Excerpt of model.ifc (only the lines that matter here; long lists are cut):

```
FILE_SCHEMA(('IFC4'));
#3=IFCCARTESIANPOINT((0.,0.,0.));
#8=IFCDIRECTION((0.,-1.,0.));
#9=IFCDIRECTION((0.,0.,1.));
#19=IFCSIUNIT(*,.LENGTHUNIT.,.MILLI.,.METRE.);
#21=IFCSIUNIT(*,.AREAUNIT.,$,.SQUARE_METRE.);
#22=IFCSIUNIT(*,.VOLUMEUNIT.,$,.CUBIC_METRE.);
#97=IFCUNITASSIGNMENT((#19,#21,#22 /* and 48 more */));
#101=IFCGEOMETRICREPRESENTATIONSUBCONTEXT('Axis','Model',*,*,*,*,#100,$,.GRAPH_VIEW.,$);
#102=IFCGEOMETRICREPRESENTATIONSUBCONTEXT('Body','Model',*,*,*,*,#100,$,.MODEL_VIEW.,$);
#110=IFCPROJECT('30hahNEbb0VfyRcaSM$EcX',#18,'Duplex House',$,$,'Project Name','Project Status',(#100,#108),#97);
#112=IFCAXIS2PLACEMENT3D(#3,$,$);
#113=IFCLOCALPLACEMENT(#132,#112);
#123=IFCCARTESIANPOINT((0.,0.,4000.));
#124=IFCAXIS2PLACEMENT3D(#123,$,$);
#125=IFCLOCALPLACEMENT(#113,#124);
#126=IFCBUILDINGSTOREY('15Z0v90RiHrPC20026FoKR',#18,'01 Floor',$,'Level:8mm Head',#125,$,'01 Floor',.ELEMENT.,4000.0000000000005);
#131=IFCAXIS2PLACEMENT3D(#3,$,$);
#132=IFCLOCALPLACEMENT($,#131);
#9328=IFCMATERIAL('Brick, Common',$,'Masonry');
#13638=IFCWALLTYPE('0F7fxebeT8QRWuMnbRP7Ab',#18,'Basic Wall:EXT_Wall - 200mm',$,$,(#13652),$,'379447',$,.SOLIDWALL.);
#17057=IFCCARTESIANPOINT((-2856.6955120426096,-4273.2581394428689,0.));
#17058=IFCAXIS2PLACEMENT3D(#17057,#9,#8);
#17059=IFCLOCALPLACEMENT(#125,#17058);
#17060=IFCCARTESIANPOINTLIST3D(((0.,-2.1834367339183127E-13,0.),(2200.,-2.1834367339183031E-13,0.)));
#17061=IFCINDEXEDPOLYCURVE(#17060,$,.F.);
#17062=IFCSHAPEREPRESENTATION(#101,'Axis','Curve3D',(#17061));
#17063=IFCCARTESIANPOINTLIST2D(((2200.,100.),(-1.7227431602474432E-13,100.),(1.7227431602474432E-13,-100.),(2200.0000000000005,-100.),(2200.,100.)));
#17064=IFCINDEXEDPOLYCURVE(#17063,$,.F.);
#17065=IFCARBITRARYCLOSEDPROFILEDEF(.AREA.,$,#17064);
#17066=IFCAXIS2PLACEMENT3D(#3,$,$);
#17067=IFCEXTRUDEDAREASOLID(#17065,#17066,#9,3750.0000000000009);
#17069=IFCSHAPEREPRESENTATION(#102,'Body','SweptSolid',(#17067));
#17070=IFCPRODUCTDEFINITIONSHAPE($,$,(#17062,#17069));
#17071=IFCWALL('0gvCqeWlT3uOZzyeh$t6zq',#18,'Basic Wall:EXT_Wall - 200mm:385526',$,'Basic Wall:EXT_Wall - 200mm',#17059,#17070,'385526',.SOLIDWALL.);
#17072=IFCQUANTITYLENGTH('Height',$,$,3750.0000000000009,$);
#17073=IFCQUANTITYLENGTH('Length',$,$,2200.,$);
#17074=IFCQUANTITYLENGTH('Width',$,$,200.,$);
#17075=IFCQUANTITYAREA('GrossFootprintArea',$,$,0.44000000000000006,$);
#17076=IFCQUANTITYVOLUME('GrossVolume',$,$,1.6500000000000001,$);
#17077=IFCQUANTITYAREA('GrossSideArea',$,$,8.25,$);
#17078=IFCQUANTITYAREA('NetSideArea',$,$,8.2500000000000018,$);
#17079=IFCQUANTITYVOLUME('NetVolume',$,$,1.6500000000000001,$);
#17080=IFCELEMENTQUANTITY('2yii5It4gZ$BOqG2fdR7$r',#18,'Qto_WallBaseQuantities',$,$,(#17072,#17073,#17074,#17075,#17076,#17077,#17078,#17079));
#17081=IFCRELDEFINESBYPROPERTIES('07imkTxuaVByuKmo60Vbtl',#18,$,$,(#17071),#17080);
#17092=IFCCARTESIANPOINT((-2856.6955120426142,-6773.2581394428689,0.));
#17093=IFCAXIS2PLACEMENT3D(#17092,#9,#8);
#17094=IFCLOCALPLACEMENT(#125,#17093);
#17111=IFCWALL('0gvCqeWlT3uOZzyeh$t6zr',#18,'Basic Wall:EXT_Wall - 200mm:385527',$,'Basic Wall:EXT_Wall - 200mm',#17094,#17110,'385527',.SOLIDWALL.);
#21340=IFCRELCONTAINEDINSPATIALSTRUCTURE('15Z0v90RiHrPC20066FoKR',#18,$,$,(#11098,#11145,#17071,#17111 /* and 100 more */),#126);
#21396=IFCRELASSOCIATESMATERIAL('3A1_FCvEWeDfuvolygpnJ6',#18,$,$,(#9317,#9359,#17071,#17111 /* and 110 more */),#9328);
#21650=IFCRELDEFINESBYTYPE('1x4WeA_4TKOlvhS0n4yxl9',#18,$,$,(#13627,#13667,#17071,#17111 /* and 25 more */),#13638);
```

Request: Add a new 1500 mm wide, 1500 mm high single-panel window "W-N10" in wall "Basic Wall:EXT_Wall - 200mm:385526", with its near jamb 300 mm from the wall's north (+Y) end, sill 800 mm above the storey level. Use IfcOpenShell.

```python
import numpy as np
import ifcopenshell
import ifcopenshell.api.feature
import ifcopenshell.api.geometry
import ifcopenshell.api.pset
import ifcopenshell.api.root
import ifcopenshell.api.spatial
import ifcopenshell.geom
import ifcopenshell.util.element
import ifcopenshell.util.placement
import ifcopenshell.util.representation
import ifcopenshell.util.shape
import ifcopenshell.util.unit

model = ifcopenshell.open("model.ifc")
unit_scale = ifcopenshell.util.unit.calculate_unit_scale(model)
area_scale = ifcopenshell.util.unit.calculate_unit_scale(model, "AREAUNIT")
volume_scale = ifcopenshell.util.unit.calculate_unit_scale(model, "VOLUMEUNIT")
settings = ifcopenshell.geom.settings()


def volume(element):
    """Net volume in cubic metres, openings subtracted."""
    shape = ifcopenshell.geom.create_shape(settings, element)
    return ifcopenshell.util.shape.get_volume(shape.geometry)


wall = model.by_guid("0gvCqeWlT3uOZzyeh$t6zq")
storey = ifcopenshell.util.element.get_container(wall, ifc_class="IfcBuildingStorey")
context = ifcopenshell.util.representation.get_context(model, "Model", "Body", "MODEL_VIEW")
before = volume(wall)

width, height, from_end, sill = 1.5, 1.5, 0.3, 0.8  # metres

# The wall runs along its own X axis, and the end named is its -X end.
wall_shape = ifcopenshell.geom.create_shape(settings, wall)
x, y, z = ifcopenshell.util.shape.get_vertices(wall_shape.geometry).T
start = x.min() + from_end
face, thickness = float(y.min()), float(y.max() - y.min())
wall_matrix = ifcopenshell.util.placement.get_local_placement(wall.ObjectPlacement)
level = ifcopenshell.util.placement.get_local_placement(storey.ObjectPlacement)[2, 3]


def in_wall(x, y):
    """Placement at x, y metres in the wall's axes, at sill height."""
    matrix = wall_matrix.copy()
    matrix[:, 3] = wall_matrix @ np.array([x / unit_scale, y / unit_scale, 0.0, 1.0])
    matrix[2, 3] = level + sill / unit_scale
    return matrix


# Opening: a box that overshoots both wall faces by 50 mm.
opening = ifcopenshell.api.root.create_entity(model, ifc_class="IfcOpeningElement", predefined_type="OPENING")
box = ifcopenshell.api.geometry.add_wall_representation(
    model, context=context, length=width, height=height, thickness=thickness + 0.1
)
ifcopenshell.api.geometry.assign_representation(model, product=opening, representation=box)
ifcopenshell.api.geometry.edit_object_placement(model, product=opening, matrix=in_wall(start, face - 0.05), is_si=False)
ifcopenshell.api.feature.add_feature(model, feature=opening, element=wall)

window = ifcopenshell.api.root.create_entity(model, ifc_class="IfcWindow", name="W-N10", predefined_type="WINDOW")
window.OverallWidth, window.OverallHeight = width / unit_scale, height / unit_scale
window.PartitioningType = "SINGLE_PANEL"
body = ifcopenshell.api.geometry.add_window_representation(
    model,
    context=context,
    overall_width=window.OverallWidth,
    overall_height=window.OverallHeight,
    partition_type="SINGLE_PANEL",
)
ifcopenshell.api.geometry.assign_representation(model, product=window, representation=body)
ifcopenshell.api.spatial.assign_container(model, products=[window], relating_structure=storey)
ifcopenshell.api.feature.add_filling(model, opening=opening, element=window)

# Centre the window in the wall's thickness.
ifcopenshell.api.geometry.edit_object_placement(model, product=window, matrix=in_wall(start, face), is_si=False)
window_shape = ifcopenshell.geom.create_shape(settings, window)
depth = ifcopenshell.util.shape.get_vertices(window_shape.geometry)[:, 1]
offset = face + thickness / 2 - (depth.min() + depth.max()) / 2
ifcopenshell.api.geometry.edit_object_placement(model, product=window, matrix=in_wall(start, offset), is_si=False)

after = volume(wall)

# Update the wall's stored quantities.
qto = model.by_id(ifcopenshell.util.element.get_pset(wall, "Qto_WallBaseQuantities", should_inherit=False)["id"])
ifcopenshell.api.pset.edit_qto(model, qto=qto, properties={
    "NetSideArea": after / thickness / area_scale,
    "NetVolume": after / volume_scale,
})

print(f"wall volume {before:.3f} -> {after:.3f} m3")

model.write("model_edited.ifc")
```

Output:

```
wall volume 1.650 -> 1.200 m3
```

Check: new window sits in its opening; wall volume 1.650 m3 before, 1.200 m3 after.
